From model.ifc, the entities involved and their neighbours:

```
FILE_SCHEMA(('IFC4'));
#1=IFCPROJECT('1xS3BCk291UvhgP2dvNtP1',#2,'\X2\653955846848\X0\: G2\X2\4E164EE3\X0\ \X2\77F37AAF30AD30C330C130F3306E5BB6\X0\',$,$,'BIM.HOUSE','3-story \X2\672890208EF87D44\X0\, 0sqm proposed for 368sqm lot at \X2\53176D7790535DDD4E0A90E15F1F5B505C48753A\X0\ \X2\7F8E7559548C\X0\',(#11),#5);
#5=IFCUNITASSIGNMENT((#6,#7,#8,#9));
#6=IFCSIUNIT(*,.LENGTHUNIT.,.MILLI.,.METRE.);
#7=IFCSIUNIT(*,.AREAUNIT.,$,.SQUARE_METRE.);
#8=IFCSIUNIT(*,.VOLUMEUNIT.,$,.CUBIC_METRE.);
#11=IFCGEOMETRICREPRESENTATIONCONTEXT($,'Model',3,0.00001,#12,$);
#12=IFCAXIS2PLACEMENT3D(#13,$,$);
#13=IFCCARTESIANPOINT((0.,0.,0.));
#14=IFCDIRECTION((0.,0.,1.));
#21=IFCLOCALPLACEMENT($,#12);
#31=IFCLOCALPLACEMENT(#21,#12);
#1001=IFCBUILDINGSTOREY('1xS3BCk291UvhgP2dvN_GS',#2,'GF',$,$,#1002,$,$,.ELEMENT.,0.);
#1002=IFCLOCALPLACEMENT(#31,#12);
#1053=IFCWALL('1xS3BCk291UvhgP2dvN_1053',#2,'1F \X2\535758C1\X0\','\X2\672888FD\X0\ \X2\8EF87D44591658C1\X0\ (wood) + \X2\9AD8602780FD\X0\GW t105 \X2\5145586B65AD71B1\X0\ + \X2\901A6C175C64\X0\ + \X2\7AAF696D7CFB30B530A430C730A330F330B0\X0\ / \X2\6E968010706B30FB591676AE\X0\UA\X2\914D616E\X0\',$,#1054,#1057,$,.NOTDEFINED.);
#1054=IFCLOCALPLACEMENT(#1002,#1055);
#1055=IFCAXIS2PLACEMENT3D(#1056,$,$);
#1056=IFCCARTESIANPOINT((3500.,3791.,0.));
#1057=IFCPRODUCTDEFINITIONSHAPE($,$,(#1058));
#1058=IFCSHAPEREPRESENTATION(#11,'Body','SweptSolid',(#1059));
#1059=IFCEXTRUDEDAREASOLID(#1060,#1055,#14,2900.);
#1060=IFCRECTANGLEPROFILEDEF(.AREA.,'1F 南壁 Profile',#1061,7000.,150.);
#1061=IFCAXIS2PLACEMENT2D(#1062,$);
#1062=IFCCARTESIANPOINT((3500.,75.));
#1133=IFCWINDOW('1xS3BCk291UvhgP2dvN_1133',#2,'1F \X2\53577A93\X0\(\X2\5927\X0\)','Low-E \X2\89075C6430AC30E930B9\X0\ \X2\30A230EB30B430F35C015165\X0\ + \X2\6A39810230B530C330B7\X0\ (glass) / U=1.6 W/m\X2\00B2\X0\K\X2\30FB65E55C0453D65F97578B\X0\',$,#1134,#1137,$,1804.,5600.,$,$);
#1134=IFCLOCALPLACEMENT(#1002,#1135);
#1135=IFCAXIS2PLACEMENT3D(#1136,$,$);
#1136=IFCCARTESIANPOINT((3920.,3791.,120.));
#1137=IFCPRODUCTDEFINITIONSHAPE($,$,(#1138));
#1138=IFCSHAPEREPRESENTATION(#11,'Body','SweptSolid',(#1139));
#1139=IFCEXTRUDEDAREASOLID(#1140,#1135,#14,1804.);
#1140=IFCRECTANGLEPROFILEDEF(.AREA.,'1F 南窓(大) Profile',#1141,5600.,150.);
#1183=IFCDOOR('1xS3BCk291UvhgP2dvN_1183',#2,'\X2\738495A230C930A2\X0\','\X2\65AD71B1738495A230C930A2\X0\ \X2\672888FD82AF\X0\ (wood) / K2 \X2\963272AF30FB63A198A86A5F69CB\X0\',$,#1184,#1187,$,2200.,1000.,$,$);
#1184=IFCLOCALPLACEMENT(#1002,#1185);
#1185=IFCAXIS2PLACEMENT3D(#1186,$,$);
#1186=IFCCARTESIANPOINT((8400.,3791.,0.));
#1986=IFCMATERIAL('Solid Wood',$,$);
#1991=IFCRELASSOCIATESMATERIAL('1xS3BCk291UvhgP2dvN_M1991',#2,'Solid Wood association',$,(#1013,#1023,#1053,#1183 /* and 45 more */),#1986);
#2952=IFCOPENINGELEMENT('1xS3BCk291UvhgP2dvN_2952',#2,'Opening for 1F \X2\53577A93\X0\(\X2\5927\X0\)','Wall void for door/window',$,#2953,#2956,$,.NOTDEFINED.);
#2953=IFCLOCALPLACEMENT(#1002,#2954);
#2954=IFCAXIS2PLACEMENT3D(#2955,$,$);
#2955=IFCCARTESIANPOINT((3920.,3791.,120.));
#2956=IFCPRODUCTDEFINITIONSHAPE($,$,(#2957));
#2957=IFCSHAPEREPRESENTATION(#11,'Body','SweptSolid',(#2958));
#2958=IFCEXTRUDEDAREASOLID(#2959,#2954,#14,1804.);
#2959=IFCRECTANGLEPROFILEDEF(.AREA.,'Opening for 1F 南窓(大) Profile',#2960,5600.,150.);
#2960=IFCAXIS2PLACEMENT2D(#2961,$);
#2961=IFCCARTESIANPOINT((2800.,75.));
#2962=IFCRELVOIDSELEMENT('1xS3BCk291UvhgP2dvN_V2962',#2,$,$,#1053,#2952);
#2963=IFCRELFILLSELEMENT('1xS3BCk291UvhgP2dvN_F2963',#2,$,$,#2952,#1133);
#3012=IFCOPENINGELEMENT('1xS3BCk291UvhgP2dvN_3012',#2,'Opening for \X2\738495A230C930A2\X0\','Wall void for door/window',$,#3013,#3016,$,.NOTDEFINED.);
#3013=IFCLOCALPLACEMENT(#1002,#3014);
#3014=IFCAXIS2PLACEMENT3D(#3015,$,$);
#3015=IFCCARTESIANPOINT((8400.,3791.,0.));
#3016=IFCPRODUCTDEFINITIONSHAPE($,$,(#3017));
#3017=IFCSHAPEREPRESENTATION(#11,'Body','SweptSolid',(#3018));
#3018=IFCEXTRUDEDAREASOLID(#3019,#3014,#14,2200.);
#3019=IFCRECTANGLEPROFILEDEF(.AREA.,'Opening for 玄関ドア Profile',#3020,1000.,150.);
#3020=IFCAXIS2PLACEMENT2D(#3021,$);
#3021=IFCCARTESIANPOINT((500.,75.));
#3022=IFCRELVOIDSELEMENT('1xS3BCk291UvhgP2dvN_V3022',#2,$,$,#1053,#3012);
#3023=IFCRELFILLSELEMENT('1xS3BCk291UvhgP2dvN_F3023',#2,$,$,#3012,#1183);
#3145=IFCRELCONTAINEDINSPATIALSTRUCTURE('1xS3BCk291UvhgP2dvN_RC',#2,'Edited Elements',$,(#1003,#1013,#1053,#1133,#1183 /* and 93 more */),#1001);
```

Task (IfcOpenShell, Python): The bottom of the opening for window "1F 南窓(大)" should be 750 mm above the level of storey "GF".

```python
import numpy as np
import ifcopenshell
import ifcopenshell.api.geometry
import ifcopenshell.geom
import ifcopenshell.util.element
import ifcopenshell.util.placement
import ifcopenshell.util.shape
import ifcopenshell.util.unit

model = ifcopenshell.open("model.ifc")
unit_scale = ifcopenshell.util.unit.calculate_unit_scale(model)

window = model.by_guid("1xS3BCk291UvhgP2dvN_1133")
opening = window.FillsVoids[0].RelatingOpeningElement
storey = ifcopenshell.util.element.get_container(window, ifc_class="IfcBuildingStorey")
level = ifcopenshell.util.placement.get_local_placement(storey.ObjectPlacement)[2, 3]

# The opening's origin need not be at the sill, so measure its lowest point.
shape = ifcopenshell.geom.create_shape(ifcopenshell.geom.settings(), opening)
bottom = ifcopenshell.util.shape.get_shape_bottom_elevation(shape, shape.geometry) / unit_scale
dz = level + 0.75 / unit_scale - bottom

shift = np.array([0.0, 0.0, dz])
# The window is not placed relative to its opening, so move both.
for product in (opening, window):
    matrix = ifcopenshell.util.placement.get_local_placement(product.ObjectPlacement)
    matrix[:3, 3] += shift
    ifcopenshell.api.geometry.edit_object_placement(model, product=product, matrix=matrix, is_si=False)

print(f"moved by {dz * unit_scale:+.3f} m")

model.write("model_v2.ifc")
```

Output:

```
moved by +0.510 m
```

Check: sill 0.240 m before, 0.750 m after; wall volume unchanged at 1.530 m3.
